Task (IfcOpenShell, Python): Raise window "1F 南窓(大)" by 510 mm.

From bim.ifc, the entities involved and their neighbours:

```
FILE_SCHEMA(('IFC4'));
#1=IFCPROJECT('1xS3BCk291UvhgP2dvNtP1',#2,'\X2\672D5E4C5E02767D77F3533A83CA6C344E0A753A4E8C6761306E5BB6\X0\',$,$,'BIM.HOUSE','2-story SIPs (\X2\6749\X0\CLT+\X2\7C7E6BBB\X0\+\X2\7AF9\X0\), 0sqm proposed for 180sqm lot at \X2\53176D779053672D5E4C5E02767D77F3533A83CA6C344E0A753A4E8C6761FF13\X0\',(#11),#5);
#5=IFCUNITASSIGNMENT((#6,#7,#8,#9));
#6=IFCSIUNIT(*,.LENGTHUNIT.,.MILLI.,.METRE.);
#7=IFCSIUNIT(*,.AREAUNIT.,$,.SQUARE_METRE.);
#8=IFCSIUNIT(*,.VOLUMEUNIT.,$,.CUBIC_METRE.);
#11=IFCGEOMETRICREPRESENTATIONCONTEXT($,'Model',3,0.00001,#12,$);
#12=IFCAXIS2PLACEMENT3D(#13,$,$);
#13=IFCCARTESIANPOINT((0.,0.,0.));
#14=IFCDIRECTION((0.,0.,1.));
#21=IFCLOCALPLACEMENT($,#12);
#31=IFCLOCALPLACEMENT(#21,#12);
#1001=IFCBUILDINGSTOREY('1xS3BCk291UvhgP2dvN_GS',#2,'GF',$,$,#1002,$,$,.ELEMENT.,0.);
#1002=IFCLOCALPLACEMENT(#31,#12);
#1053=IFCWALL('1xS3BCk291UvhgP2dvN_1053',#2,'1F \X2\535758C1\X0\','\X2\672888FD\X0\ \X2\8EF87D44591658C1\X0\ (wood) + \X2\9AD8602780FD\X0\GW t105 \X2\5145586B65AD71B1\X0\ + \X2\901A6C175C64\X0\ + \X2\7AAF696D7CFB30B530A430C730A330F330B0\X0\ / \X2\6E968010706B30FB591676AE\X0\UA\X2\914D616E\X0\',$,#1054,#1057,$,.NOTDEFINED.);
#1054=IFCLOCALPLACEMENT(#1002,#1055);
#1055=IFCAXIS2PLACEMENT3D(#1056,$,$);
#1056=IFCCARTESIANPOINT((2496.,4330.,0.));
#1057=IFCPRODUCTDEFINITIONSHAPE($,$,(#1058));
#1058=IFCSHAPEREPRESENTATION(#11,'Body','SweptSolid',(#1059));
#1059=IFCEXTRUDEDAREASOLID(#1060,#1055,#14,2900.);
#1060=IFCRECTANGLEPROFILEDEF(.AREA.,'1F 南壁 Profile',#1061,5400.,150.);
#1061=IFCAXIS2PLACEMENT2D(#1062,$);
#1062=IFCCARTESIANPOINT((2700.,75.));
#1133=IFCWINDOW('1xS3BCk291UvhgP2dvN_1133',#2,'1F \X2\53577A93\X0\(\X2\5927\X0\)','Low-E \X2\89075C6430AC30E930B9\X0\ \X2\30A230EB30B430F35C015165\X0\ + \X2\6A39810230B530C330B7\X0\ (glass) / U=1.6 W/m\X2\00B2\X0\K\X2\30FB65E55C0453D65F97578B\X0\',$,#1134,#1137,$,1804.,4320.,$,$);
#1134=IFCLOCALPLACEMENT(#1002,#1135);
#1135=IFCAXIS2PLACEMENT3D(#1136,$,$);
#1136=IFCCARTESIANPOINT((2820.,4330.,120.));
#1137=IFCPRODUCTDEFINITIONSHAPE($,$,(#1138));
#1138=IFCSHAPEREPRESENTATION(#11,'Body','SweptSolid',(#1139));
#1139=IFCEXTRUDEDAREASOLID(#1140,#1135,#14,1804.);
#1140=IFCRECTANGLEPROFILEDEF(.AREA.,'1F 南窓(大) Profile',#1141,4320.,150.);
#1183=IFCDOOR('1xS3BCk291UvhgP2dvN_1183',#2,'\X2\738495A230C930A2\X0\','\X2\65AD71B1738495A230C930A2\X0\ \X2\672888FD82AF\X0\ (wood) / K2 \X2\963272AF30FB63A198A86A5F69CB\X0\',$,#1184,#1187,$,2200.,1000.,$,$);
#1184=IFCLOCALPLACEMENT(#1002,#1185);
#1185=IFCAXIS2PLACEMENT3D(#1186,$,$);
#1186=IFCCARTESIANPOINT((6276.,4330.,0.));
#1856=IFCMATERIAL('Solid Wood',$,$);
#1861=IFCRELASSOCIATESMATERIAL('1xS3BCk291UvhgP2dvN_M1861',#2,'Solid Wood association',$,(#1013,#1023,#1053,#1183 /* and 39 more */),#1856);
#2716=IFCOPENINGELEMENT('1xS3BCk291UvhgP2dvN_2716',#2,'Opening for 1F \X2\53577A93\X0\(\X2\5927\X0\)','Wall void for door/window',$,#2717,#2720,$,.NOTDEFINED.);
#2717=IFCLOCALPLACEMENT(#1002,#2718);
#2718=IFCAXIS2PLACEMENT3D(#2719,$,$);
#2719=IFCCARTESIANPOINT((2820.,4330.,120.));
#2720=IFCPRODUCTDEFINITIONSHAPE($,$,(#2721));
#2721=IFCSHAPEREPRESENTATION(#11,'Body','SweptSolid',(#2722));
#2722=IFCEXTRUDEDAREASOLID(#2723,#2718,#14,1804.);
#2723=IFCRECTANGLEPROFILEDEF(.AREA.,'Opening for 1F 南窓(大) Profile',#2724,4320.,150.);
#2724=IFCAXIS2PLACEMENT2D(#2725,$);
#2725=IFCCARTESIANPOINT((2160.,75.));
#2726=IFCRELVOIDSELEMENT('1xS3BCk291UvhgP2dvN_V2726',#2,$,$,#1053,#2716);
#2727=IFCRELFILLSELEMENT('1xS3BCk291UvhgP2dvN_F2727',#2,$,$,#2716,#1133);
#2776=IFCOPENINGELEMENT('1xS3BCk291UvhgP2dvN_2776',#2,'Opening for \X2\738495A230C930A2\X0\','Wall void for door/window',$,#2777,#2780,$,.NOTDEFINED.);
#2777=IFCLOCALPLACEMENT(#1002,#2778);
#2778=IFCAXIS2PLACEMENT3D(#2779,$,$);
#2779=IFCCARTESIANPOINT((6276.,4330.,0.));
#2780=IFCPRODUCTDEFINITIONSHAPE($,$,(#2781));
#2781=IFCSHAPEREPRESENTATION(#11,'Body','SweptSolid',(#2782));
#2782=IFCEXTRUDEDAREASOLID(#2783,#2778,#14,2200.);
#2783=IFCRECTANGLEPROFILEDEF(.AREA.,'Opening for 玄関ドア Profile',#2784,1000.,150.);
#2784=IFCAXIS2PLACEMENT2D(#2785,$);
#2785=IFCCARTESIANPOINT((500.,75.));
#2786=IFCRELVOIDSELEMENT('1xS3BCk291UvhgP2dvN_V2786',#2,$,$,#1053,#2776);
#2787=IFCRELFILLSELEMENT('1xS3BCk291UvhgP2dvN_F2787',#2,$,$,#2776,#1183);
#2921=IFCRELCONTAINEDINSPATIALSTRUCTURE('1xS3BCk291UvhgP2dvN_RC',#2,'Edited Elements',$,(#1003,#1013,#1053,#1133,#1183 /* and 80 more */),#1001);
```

```python
import numpy as np
import ifcopenshell
import ifcopenshell.api.geometry
import ifcopenshell.util.placement
import ifcopenshell.util.unit

model = ifcopenshell.open("bim.ifc")
unit_scale = ifcopenshell.util.unit.calculate_unit_scale(model)

window = model.by_guid("1xS3BCk291UvhgP2dvN_1133")
opening = window.FillsVoids[0].RelatingOpeningElement
dz = 510.0

shift = np.array([0.0, 0.0, dz])
# The window is not placed relative to its opening, so move both.
for product in (opening, window):
    matrix = ifcopenshell.util.placement.get_local_placement(product.ObjectPlacement)
    matrix[:3, 3] += shift
    ifcopenshell.api.geometry.edit_object_placement(model, product=product, matrix=matrix, is_si=False)

print(f"moved by {dz * unit_scale:+.3f} m")

model.write("bim_updated.ifc")
```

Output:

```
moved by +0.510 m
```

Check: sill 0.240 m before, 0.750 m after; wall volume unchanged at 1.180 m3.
